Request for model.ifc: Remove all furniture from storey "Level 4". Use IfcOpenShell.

First a look at what the model holds.

```python
import ifcopenshell
import ifcopenshell.util.element

model = ifcopenshell.open("model.ifc")
print(model.schema)
storey = next(s for s in model.by_type("IfcBuildingStorey") if s.Name == "Level 4")
furniture = [e for e in ifcopenshell.util.element.get_decomposition(storey) if e.is_a("IfcFurnishingElement")]
seen = {}
for e in furniture:
    element_type = ifcopenshell.util.element.get_type(e)
    name = element_type.Name if element_type not in (None, e) else None
    seen[name] = seen.get(name, 0) + 1
for name, count in sorted(seen.items(), key=str):
    print(count, "x", name)
```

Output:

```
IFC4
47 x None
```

```python
import ifcopenshell
import ifcopenshell.api.root
import ifcopenshell.util.element

model = ifcopenshell.open("model.ifc")

storey = next(s for s in model.by_type("IfcBuildingStorey") if s.Name == "Level 4")
furniture = [e for e in ifcopenshell.util.element.get_decomposition(storey) if e.is_a("IfcFurnishingElement")]

for e in furniture:
    ifcopenshell.api.root.remove_product(model, product=e)
print(len(furniture), "removed")

model.write("model_v2.ifc")
```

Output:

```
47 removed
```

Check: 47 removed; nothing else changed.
